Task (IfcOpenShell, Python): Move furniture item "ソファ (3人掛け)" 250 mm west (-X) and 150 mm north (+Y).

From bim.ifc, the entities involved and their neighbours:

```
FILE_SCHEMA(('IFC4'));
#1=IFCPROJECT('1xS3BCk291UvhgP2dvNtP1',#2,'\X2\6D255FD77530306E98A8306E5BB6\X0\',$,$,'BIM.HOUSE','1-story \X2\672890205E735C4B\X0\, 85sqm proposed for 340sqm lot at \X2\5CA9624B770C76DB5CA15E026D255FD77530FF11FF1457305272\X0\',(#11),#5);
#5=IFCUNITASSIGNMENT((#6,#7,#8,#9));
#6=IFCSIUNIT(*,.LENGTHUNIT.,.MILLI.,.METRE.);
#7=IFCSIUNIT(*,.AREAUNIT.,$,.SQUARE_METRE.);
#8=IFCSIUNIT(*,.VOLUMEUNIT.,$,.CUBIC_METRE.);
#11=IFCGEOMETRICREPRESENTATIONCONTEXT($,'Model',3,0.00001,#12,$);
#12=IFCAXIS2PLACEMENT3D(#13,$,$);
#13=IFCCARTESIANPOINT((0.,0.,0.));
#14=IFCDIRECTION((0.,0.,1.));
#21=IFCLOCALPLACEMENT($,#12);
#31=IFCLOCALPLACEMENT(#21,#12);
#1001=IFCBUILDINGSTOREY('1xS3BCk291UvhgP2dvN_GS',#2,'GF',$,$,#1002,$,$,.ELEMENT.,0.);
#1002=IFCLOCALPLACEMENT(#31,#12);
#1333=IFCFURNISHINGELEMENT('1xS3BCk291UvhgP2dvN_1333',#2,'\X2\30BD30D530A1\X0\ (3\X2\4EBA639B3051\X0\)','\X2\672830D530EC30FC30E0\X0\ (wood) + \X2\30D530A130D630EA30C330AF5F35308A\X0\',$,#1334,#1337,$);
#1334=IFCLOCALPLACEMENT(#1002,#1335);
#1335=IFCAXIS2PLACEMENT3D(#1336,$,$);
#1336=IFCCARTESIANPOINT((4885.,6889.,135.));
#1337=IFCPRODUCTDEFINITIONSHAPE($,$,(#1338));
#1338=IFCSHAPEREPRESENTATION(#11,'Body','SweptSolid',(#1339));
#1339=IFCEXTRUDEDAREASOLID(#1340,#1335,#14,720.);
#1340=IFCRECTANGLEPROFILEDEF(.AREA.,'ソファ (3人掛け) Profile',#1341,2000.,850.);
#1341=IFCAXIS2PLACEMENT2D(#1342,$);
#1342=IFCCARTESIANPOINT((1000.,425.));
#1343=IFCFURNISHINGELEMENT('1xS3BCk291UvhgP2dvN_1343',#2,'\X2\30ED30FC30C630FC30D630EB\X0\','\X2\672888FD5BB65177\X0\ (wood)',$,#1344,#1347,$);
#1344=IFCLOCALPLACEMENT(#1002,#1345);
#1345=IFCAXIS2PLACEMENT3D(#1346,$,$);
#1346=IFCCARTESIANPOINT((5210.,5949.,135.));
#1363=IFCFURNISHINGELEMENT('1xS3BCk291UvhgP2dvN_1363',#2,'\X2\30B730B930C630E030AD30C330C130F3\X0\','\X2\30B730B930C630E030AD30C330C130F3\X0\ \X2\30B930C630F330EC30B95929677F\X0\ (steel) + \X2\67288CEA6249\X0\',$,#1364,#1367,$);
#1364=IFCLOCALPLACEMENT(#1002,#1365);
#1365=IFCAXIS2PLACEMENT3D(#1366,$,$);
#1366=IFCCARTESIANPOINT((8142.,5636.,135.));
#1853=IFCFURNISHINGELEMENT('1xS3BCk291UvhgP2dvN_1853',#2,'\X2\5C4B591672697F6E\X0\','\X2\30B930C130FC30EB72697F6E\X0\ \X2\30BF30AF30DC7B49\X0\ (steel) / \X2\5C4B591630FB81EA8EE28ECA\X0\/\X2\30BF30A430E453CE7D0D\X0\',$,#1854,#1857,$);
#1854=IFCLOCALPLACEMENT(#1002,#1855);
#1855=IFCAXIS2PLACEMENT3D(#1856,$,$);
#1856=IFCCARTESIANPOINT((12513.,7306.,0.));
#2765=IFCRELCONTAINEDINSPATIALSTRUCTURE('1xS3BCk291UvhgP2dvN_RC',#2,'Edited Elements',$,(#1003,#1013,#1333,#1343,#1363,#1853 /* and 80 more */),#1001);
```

```python
import ifcopenshell
import ifcopenshell.api.geometry
import ifcopenshell.util.placement

model = ifcopenshell.open("bim.ifc")

item = model.by_guid("1xS3BCk291UvhgP2dvN_1333")
matrix = ifcopenshell.util.placement.get_local_placement(item.ObjectPlacement)
matrix[0, 3] -= 250.0
matrix[1, 3] += 150.0
ifcopenshell.api.geometry.edit_object_placement(model, product=item, matrix=matrix, is_si=False)

print(ifcopenshell.util.placement.get_local_placement(item.ObjectPlacement).round(3) + 0.0)

model.write("bim_updated.ifc")
```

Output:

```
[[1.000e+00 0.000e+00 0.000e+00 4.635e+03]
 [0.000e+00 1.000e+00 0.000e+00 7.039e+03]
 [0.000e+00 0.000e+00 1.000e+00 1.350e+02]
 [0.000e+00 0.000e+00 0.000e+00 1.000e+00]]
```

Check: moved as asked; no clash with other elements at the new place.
